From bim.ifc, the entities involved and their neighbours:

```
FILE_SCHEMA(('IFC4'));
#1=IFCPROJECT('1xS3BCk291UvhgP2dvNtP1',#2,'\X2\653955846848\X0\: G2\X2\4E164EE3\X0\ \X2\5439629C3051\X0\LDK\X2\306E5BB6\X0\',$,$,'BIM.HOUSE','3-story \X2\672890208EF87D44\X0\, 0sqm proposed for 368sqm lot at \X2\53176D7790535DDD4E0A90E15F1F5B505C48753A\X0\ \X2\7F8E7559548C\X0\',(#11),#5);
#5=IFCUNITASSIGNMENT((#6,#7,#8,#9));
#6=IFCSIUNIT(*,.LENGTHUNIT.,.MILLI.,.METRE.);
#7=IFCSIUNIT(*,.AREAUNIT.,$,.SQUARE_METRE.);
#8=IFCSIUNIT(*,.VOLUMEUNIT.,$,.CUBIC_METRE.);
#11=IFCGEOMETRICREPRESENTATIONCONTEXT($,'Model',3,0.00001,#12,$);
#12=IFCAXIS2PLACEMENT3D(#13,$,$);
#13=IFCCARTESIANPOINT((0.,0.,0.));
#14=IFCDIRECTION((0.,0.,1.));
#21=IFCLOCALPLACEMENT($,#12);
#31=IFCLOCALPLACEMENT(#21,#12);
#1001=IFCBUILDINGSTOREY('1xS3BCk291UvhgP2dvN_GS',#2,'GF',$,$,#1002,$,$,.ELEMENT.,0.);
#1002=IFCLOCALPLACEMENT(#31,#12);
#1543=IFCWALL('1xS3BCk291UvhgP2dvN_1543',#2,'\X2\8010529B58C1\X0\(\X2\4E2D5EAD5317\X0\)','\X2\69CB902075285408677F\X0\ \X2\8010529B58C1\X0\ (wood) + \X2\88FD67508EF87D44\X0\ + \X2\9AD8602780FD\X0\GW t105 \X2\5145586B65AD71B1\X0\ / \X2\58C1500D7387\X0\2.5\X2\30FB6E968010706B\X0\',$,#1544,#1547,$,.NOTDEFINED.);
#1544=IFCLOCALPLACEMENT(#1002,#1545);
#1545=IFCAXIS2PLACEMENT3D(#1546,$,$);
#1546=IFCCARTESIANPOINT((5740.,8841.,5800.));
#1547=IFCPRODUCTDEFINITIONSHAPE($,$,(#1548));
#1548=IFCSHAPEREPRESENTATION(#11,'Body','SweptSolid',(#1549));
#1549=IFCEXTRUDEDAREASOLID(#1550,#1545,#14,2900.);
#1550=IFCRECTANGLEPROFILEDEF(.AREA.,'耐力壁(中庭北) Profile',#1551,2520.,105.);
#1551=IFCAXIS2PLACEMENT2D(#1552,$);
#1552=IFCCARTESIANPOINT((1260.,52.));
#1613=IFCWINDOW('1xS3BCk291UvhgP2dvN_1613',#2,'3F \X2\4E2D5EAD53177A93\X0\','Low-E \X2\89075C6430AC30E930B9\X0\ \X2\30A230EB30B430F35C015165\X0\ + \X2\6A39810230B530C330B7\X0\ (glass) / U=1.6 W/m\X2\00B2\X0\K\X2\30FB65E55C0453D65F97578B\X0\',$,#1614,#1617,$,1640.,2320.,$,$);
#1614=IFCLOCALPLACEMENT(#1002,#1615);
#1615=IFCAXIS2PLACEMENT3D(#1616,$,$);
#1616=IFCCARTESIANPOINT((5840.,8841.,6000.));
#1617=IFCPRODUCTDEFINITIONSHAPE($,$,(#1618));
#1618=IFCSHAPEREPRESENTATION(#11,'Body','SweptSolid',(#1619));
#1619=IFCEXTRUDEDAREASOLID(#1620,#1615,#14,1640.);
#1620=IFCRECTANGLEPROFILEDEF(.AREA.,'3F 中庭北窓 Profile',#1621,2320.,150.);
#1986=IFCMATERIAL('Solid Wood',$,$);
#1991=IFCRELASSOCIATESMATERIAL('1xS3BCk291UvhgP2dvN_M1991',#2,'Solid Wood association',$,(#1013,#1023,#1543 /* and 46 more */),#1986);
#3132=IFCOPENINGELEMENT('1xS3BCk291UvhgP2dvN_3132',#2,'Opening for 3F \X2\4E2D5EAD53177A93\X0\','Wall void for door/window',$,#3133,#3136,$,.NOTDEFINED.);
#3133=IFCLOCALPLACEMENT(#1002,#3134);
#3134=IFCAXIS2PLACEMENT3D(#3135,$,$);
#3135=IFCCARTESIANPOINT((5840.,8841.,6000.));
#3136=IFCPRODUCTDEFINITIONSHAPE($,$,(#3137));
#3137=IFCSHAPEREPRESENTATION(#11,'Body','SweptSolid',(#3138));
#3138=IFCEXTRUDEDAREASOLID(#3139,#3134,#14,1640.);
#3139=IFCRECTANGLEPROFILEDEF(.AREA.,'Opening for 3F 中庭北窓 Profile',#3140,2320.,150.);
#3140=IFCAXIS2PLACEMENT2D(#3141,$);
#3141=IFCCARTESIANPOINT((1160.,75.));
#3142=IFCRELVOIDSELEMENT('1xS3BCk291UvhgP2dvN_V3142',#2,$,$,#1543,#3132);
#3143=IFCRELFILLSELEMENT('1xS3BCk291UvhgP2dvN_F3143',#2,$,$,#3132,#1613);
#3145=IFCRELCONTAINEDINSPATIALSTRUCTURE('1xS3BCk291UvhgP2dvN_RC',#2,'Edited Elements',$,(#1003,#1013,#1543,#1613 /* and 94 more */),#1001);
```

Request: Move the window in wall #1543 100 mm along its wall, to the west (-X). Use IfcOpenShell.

```python
import ifcopenshell
import ifcopenshell.api.geometry
import ifcopenshell.util.placement
import ifcopenshell.util.unit

model = ifcopenshell.open("bim.ifc")
unit_scale = ifcopenshell.util.unit.calculate_unit_scale(model)

window = model.by_guid("1xS3BCk291UvhgP2dvN_1613")
opening = window.FillsVoids[0].RelatingOpeningElement
wall = opening.VoidsElements[0].RelatingBuildingElement

wall_matrix = ifcopenshell.util.placement.get_local_placement(wall.ObjectPlacement)
shift = wall_matrix[:3, 0] * -0.1 / unit_scale
before = ifcopenshell.util.placement.get_local_placement(window.ObjectPlacement)[:3, 3].copy()

# The window is not placed relative to its opening, so move both.
for product in (opening, window):
    matrix = ifcopenshell.util.placement.get_local_placement(product.ObjectPlacement)
    matrix[:3, 3] += shift
    ifcopenshell.api.geometry.edit_object_placement(model, product=product, matrix=matrix, is_si=False)

after = ifcopenshell.util.placement.get_local_placement(window.ObjectPlacement)[:3, 3]
print("window moved by", (after - before).round(3) + 0.0)

model.write("bim_edited.ifc")
```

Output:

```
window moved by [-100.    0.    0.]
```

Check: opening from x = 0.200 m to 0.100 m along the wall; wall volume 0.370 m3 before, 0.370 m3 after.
